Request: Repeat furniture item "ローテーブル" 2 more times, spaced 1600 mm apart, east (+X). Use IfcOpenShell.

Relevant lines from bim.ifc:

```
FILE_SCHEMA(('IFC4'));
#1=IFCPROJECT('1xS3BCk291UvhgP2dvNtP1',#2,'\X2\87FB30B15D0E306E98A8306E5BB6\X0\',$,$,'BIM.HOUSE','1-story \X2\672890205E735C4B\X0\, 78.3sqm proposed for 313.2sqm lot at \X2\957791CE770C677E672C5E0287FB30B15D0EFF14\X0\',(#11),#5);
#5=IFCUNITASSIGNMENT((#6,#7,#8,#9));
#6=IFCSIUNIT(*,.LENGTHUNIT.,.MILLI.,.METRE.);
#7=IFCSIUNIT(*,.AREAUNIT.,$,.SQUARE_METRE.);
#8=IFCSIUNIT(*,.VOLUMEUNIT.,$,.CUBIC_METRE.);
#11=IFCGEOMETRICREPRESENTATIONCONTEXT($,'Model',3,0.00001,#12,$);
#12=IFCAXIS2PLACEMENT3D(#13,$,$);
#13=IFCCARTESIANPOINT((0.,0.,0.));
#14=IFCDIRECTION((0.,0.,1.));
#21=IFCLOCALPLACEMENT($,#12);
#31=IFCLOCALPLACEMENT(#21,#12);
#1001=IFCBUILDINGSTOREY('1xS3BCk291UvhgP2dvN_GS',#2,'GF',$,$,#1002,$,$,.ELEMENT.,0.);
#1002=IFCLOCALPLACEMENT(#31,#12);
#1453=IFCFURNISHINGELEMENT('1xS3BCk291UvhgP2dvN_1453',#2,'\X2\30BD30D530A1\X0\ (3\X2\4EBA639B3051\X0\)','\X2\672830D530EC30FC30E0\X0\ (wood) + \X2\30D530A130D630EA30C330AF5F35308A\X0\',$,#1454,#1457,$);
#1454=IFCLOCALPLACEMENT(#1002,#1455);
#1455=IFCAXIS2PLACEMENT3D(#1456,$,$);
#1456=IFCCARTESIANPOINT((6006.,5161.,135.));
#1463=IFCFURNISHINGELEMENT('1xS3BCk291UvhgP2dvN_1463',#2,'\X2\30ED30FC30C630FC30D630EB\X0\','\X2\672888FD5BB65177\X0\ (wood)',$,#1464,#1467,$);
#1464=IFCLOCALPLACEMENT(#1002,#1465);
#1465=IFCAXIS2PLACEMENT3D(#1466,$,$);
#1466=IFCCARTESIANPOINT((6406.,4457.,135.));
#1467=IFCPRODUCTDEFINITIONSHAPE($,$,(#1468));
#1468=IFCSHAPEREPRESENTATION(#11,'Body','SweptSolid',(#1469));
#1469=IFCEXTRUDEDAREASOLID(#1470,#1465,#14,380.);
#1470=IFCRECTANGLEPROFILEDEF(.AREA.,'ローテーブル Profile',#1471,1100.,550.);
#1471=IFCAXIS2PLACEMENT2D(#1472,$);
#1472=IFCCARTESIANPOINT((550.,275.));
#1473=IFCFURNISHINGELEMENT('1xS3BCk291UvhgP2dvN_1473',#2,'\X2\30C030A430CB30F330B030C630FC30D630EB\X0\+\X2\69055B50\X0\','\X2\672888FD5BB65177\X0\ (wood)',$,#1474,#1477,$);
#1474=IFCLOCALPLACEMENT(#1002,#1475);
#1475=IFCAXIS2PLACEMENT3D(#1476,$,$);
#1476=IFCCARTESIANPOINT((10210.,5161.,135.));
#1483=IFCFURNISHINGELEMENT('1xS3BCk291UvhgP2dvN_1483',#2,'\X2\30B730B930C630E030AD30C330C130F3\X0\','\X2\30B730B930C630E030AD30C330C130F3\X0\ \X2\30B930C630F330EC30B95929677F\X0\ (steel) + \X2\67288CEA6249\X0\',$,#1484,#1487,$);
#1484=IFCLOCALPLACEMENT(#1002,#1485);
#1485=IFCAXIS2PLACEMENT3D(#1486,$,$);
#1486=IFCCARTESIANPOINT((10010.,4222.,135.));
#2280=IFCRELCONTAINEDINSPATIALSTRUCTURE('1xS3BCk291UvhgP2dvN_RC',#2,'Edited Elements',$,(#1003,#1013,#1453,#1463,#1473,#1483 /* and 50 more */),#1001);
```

```python
import numpy as np
import ifcopenshell
import ifcopenshell.api.geometry
import ifcopenshell.api.root
import ifcopenshell.util.element
import ifcopenshell.util.placement

model = ifcopenshell.open("bim.ifc")


def reuse_history(source, copy):
    """copy_class also copies each property set's owner history, people and application; keep the originals."""
    for rel in copy.IsDefinedBy:
        if rel.is_a("IfcRelDefinesByProperties") and (history := rel.RelatingPropertyDefinition.OwnerHistory):
            rel.RelatingPropertyDefinition.OwnerHistory = source.OwnerHistory
            ifcopenshell.util.element.remove_deep2(model, history)


source = model.by_guid("1xS3BCk291UvhgP2dvN_1463")
base = ifcopenshell.util.placement.get_local_placement(source.ObjectPlacement)
step = np.array([1.0, 0.0, 0.0]) * 1600.0

for i in range(1, 3):
    copy = ifcopenshell.api.root.copy_class(model, product=source)
    copy.Representation = ifcopenshell.util.element.copy_deep(
        model, source.Representation, exclude=["IfcGeometricRepresentationContext", "IfcRepresentationMap"]
    )
    reuse_history(source, copy)
    matrix = base.copy()
    matrix[:3, 3] += i * step
    print("added at", matrix[:3, 3].round(3) + 0.0)
    ifcopenshell.api.geometry.edit_object_placement(model, product=copy, matrix=matrix, is_si=False)

model.write("bim_rev.ifc")
```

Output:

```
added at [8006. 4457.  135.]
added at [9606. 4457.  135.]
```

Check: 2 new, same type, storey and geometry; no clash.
